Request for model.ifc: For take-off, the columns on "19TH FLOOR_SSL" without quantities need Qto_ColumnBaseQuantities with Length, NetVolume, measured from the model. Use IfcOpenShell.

First a look at what the model holds.

```python
import ifcopenshell
import ifcopenshell.util.element
import ifcopenshell.util.unit

model = ifcopenshell.open("model.ifc")
print(model.schema)
for unit_type in ("LENGTHUNIT", "AREAUNIT", "VOLUMEUNIT"):
    print(unit_type, ifcopenshell.util.unit.calculate_unit_scale(model, unit_type))
storey = next(s for s in model.by_type("IfcBuildingStorey") if s.Name == "19TH FLOOR_SSL")
columns = [e for e in ifcopenshell.util.element.get_decomposition(storey) if e.is_a("IfcColumn")]
for e in sorted(columns, key=lambda e: e.id()):
    print(e.id(), e.is_a(), e.Name, list(ifcopenshell.util.element.get_psets(e, qtos_only=True)), sep=" | ")
```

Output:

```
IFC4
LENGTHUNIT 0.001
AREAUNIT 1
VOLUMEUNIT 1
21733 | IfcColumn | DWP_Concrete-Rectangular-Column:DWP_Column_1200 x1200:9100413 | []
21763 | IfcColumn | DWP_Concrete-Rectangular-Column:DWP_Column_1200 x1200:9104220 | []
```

```python
import ifcopenshell
import ifcopenshell.api.pset
import ifcopenshell.geom
import ifcopenshell.util.element
import ifcopenshell.util.shape
import ifcopenshell.util.unit

model = ifcopenshell.open("model.ifc")
unit_scale = ifcopenshell.util.unit.calculate_unit_scale(model)
volume_scale = ifcopenshell.util.unit.calculate_unit_scale(model, "VOLUMEUNIT")
settings = ifcopenshell.geom.settings()

storey = next(s for s in model.by_type("IfcBuildingStorey") if s.Name == "19TH FLOOR_SSL")
columns = [e for e in ifcopenshell.util.element.get_decomposition(storey) if e.is_a("IfcColumn")]

for e in sorted(columns, key=lambda e: e.id()):
    if ifcopenshell.util.element.get_psets(e, qtos_only=True, should_inherit=False):
        continue
    # Geometry comes back in metres, in the element's own axes.
    shape = ifcopenshell.geom.create_shape(settings, e)
    values = {
        "Length": ifcopenshell.util.shape.get_z(shape.geometry) / unit_scale,
        "NetVolume": ifcopenshell.util.shape.get_volume(shape.geometry) / volume_scale,
    }
    qto = ifcopenshell.api.pset.add_qto(model, product=e, name="Qto_ColumnBaseQuantities")
    ifcopenshell.api.pset.edit_qto(model, qto=qto, properties=values)
    print(e.id(), {k: round(v, 3) for k, v in values.items()})

model.write("model_v2.ifc")
```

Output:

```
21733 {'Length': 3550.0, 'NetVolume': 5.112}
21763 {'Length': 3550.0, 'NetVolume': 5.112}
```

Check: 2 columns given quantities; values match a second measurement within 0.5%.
